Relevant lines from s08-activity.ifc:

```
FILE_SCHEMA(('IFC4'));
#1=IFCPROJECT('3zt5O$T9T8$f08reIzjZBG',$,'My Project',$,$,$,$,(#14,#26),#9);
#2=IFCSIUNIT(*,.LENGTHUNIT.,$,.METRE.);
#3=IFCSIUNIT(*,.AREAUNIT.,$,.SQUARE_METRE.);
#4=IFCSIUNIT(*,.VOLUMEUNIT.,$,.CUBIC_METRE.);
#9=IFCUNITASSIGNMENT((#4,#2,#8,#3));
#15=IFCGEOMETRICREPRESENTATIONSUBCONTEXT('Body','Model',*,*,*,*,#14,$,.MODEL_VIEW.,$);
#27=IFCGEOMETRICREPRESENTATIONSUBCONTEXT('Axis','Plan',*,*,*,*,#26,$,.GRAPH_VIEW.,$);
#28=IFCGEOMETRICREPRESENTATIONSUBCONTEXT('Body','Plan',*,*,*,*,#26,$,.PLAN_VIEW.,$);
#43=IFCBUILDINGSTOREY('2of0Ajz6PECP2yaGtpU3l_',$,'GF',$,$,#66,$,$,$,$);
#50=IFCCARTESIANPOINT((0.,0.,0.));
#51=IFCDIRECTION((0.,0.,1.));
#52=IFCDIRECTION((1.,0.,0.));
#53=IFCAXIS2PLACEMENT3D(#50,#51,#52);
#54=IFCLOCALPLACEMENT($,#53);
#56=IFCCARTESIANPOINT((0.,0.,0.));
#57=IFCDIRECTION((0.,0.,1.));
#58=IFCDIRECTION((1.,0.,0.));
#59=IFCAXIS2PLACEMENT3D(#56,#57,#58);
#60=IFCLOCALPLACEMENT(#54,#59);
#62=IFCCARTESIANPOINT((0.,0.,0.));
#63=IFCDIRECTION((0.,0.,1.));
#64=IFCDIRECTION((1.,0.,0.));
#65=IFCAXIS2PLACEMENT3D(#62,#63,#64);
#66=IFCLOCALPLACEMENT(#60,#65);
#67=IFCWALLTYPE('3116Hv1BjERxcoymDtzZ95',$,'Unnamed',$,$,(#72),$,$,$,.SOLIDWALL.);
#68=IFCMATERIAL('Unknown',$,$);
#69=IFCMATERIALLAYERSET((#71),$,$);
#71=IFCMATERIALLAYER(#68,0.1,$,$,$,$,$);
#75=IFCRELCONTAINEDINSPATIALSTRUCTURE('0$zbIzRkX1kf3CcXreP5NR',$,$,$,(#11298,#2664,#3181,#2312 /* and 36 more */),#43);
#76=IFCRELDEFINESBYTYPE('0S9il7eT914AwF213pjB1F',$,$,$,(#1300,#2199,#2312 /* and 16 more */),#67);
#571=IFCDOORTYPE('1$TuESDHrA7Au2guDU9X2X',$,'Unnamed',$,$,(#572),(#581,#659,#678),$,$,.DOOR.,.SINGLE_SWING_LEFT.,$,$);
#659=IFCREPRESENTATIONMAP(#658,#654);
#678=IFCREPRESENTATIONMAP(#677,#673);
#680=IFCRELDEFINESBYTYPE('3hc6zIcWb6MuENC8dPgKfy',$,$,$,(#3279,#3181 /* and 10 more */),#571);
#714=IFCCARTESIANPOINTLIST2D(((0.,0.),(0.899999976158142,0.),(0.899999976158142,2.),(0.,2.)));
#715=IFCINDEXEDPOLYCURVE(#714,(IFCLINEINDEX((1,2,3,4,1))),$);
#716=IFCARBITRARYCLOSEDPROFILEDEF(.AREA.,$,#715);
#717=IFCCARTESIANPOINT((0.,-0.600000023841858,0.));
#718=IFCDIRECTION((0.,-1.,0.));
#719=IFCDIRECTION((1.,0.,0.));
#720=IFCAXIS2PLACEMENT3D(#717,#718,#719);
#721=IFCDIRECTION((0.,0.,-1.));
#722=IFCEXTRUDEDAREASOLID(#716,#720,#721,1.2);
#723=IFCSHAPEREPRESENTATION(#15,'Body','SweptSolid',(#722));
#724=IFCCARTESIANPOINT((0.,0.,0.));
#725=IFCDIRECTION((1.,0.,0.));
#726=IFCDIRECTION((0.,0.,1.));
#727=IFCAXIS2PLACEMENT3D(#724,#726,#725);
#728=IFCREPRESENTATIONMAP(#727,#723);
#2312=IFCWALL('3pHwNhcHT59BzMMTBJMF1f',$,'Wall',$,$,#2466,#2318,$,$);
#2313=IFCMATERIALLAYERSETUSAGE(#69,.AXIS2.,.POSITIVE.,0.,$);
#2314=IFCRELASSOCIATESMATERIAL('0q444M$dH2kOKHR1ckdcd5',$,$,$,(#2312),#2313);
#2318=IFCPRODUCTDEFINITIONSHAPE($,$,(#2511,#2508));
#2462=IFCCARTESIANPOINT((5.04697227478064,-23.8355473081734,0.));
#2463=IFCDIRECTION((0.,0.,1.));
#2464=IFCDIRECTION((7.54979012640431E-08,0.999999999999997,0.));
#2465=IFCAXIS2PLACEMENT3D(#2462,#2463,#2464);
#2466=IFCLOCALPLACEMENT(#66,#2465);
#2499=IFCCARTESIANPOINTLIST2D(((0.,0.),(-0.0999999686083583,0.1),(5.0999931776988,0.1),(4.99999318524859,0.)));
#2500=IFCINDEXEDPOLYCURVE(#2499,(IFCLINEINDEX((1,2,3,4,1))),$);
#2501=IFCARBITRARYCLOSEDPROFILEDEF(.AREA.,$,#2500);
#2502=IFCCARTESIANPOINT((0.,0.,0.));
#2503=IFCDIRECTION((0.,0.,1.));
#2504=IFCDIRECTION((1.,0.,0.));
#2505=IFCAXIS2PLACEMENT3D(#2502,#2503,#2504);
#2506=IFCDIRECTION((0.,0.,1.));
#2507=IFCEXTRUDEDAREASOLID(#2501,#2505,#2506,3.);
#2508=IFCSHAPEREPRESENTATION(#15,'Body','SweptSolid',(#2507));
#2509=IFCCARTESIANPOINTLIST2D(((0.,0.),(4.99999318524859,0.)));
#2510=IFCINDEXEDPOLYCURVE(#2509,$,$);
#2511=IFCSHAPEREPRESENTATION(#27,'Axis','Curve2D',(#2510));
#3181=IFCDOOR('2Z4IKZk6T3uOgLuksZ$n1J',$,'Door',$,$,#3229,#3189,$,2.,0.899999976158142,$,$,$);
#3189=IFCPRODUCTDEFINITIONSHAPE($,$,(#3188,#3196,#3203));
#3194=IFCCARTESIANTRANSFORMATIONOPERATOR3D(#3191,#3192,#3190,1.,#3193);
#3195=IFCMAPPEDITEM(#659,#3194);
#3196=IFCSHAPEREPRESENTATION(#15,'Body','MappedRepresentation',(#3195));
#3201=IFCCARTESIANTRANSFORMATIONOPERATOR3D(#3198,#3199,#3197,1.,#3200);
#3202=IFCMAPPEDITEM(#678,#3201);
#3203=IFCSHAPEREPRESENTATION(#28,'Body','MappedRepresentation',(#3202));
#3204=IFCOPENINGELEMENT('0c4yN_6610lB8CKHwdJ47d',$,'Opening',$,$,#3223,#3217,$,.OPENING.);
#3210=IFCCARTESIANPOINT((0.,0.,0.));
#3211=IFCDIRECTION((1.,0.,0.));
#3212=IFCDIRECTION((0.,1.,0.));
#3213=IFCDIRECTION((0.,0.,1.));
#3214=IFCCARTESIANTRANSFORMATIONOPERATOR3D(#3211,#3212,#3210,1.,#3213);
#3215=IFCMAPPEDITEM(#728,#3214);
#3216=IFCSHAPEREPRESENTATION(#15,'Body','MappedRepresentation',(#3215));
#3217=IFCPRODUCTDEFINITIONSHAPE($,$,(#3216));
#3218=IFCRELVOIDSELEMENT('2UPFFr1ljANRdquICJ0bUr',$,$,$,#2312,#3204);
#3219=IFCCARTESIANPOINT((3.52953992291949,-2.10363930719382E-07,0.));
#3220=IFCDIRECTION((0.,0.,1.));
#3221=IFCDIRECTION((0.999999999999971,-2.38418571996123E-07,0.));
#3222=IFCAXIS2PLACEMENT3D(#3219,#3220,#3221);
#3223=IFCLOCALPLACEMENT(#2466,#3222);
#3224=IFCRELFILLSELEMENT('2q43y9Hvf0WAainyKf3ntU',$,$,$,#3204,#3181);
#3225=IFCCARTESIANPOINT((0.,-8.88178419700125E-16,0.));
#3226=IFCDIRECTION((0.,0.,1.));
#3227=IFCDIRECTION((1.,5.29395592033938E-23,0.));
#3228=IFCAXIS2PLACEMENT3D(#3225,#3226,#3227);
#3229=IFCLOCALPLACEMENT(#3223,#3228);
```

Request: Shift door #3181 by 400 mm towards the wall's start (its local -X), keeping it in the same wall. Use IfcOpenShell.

```python
import ifcopenshell
import ifcopenshell.api.geometry
import ifcopenshell.util.placement

model = ifcopenshell.open("s08-activity.ifc")

door = model.by_guid("2Z4IKZk6T3uOgLuksZ$n1J")
opening = door.FillsVoids[0].RelatingOpeningElement
wall = opening.VoidsElements[0].RelatingBuildingElement

wall_matrix = ifcopenshell.util.placement.get_local_placement(wall.ObjectPlacement)
shift = wall_matrix[:3, 0] * -0.4
before = ifcopenshell.util.placement.get_local_placement(door.ObjectPlacement)[:3, 3].copy()

# The door is placed relative to its opening, so it follows when the opening moves.
matrix = ifcopenshell.util.placement.get_local_placement(opening.ObjectPlacement)
matrix[:3, 3] += shift
ifcopenshell.api.geometry.edit_object_placement(
    model, product=opening, matrix=matrix, is_si=False, should_transform_children=True
)

after = ifcopenshell.util.placement.get_local_placement(door.ObjectPlacement)[:3, 3]
print("door moved by", (after - before).round(3) + 0.0)

model.write("s08-activity-out.ifc")
```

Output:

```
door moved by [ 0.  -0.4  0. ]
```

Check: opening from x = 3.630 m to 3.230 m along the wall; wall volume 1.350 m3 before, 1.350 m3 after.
